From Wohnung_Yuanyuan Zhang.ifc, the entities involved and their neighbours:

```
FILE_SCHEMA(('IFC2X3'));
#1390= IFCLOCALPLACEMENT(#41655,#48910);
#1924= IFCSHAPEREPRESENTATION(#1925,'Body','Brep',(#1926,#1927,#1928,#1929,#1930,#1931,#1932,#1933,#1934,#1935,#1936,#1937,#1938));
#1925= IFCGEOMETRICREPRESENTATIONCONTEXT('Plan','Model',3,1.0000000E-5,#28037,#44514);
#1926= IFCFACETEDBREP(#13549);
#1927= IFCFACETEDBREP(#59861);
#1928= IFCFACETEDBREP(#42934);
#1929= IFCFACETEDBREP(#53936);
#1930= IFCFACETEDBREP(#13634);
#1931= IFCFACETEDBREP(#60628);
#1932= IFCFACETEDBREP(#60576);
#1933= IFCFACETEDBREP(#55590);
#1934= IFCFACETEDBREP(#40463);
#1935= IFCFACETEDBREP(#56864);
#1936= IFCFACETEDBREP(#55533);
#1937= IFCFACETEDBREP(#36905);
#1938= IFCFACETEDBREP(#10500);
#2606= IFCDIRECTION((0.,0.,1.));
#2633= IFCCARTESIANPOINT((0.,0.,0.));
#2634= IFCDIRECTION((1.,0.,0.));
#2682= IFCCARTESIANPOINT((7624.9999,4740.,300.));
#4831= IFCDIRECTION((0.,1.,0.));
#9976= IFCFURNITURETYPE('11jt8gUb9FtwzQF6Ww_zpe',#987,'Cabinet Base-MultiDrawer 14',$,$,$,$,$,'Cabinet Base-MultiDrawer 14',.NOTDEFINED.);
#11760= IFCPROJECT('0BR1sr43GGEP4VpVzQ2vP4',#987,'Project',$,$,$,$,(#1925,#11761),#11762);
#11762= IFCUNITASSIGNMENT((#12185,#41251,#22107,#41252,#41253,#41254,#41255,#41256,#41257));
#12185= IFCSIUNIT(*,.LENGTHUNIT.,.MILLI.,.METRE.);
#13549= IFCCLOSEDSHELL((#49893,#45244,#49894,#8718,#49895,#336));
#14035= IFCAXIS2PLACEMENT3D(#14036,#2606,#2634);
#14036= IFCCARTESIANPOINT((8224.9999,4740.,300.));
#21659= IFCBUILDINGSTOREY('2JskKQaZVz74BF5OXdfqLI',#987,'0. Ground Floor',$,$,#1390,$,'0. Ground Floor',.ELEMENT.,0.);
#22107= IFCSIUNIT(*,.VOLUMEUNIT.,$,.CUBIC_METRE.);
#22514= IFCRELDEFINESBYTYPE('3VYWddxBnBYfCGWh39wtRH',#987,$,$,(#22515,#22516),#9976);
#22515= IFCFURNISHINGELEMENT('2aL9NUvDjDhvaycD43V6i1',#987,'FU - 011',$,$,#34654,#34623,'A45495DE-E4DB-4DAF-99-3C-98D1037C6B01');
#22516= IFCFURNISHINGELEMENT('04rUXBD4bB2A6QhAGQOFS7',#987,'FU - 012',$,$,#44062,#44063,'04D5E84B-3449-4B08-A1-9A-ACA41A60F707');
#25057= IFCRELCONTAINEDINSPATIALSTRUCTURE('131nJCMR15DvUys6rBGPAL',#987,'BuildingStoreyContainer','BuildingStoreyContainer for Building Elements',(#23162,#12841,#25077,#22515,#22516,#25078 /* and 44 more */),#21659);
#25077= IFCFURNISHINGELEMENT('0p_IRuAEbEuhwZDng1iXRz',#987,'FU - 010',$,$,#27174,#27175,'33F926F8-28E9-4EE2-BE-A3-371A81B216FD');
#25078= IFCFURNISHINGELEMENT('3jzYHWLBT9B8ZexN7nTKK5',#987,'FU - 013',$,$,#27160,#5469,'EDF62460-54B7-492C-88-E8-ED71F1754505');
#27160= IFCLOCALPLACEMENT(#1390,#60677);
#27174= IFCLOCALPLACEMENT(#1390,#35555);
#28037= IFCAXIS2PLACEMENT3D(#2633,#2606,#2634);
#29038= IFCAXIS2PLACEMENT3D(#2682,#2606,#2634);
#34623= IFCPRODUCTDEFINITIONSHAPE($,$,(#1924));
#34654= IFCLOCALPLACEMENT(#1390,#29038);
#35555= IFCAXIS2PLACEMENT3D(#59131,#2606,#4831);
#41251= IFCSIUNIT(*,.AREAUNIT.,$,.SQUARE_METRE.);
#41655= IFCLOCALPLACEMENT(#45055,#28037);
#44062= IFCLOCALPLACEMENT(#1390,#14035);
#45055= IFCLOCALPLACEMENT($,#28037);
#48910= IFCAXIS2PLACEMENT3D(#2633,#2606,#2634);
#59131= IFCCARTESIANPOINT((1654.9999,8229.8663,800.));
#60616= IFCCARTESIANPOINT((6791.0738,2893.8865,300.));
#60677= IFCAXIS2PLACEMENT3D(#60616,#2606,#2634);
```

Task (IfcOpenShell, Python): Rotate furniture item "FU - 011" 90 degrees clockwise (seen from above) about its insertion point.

```python
import ifcopenshell
import ifcopenshell.api.geometry
import ifcopenshell.util.placement

model = ifcopenshell.open("Wohnung_Yuanyuan Zhang.ifc")

item = model.by_id(22515)
matrix = ifcopenshell.util.placement.get_local_placement(item.ObjectPlacement)
matrix = matrix @ ifcopenshell.util.placement.rotation(-90, "Z")
ifcopenshell.api.geometry.edit_object_placement(model, product=item, matrix=matrix, is_si=False)

print(ifcopenshell.util.placement.get_local_placement(item.ObjectPlacement).round(3) + 0.0)

model.write("Wohnung_Yuanyuan Zhang_updated.ifc")
```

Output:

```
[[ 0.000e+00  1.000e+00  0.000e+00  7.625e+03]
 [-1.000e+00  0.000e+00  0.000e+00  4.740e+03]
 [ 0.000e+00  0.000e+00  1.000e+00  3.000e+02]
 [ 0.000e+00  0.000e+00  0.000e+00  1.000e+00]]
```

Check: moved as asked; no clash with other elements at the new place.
